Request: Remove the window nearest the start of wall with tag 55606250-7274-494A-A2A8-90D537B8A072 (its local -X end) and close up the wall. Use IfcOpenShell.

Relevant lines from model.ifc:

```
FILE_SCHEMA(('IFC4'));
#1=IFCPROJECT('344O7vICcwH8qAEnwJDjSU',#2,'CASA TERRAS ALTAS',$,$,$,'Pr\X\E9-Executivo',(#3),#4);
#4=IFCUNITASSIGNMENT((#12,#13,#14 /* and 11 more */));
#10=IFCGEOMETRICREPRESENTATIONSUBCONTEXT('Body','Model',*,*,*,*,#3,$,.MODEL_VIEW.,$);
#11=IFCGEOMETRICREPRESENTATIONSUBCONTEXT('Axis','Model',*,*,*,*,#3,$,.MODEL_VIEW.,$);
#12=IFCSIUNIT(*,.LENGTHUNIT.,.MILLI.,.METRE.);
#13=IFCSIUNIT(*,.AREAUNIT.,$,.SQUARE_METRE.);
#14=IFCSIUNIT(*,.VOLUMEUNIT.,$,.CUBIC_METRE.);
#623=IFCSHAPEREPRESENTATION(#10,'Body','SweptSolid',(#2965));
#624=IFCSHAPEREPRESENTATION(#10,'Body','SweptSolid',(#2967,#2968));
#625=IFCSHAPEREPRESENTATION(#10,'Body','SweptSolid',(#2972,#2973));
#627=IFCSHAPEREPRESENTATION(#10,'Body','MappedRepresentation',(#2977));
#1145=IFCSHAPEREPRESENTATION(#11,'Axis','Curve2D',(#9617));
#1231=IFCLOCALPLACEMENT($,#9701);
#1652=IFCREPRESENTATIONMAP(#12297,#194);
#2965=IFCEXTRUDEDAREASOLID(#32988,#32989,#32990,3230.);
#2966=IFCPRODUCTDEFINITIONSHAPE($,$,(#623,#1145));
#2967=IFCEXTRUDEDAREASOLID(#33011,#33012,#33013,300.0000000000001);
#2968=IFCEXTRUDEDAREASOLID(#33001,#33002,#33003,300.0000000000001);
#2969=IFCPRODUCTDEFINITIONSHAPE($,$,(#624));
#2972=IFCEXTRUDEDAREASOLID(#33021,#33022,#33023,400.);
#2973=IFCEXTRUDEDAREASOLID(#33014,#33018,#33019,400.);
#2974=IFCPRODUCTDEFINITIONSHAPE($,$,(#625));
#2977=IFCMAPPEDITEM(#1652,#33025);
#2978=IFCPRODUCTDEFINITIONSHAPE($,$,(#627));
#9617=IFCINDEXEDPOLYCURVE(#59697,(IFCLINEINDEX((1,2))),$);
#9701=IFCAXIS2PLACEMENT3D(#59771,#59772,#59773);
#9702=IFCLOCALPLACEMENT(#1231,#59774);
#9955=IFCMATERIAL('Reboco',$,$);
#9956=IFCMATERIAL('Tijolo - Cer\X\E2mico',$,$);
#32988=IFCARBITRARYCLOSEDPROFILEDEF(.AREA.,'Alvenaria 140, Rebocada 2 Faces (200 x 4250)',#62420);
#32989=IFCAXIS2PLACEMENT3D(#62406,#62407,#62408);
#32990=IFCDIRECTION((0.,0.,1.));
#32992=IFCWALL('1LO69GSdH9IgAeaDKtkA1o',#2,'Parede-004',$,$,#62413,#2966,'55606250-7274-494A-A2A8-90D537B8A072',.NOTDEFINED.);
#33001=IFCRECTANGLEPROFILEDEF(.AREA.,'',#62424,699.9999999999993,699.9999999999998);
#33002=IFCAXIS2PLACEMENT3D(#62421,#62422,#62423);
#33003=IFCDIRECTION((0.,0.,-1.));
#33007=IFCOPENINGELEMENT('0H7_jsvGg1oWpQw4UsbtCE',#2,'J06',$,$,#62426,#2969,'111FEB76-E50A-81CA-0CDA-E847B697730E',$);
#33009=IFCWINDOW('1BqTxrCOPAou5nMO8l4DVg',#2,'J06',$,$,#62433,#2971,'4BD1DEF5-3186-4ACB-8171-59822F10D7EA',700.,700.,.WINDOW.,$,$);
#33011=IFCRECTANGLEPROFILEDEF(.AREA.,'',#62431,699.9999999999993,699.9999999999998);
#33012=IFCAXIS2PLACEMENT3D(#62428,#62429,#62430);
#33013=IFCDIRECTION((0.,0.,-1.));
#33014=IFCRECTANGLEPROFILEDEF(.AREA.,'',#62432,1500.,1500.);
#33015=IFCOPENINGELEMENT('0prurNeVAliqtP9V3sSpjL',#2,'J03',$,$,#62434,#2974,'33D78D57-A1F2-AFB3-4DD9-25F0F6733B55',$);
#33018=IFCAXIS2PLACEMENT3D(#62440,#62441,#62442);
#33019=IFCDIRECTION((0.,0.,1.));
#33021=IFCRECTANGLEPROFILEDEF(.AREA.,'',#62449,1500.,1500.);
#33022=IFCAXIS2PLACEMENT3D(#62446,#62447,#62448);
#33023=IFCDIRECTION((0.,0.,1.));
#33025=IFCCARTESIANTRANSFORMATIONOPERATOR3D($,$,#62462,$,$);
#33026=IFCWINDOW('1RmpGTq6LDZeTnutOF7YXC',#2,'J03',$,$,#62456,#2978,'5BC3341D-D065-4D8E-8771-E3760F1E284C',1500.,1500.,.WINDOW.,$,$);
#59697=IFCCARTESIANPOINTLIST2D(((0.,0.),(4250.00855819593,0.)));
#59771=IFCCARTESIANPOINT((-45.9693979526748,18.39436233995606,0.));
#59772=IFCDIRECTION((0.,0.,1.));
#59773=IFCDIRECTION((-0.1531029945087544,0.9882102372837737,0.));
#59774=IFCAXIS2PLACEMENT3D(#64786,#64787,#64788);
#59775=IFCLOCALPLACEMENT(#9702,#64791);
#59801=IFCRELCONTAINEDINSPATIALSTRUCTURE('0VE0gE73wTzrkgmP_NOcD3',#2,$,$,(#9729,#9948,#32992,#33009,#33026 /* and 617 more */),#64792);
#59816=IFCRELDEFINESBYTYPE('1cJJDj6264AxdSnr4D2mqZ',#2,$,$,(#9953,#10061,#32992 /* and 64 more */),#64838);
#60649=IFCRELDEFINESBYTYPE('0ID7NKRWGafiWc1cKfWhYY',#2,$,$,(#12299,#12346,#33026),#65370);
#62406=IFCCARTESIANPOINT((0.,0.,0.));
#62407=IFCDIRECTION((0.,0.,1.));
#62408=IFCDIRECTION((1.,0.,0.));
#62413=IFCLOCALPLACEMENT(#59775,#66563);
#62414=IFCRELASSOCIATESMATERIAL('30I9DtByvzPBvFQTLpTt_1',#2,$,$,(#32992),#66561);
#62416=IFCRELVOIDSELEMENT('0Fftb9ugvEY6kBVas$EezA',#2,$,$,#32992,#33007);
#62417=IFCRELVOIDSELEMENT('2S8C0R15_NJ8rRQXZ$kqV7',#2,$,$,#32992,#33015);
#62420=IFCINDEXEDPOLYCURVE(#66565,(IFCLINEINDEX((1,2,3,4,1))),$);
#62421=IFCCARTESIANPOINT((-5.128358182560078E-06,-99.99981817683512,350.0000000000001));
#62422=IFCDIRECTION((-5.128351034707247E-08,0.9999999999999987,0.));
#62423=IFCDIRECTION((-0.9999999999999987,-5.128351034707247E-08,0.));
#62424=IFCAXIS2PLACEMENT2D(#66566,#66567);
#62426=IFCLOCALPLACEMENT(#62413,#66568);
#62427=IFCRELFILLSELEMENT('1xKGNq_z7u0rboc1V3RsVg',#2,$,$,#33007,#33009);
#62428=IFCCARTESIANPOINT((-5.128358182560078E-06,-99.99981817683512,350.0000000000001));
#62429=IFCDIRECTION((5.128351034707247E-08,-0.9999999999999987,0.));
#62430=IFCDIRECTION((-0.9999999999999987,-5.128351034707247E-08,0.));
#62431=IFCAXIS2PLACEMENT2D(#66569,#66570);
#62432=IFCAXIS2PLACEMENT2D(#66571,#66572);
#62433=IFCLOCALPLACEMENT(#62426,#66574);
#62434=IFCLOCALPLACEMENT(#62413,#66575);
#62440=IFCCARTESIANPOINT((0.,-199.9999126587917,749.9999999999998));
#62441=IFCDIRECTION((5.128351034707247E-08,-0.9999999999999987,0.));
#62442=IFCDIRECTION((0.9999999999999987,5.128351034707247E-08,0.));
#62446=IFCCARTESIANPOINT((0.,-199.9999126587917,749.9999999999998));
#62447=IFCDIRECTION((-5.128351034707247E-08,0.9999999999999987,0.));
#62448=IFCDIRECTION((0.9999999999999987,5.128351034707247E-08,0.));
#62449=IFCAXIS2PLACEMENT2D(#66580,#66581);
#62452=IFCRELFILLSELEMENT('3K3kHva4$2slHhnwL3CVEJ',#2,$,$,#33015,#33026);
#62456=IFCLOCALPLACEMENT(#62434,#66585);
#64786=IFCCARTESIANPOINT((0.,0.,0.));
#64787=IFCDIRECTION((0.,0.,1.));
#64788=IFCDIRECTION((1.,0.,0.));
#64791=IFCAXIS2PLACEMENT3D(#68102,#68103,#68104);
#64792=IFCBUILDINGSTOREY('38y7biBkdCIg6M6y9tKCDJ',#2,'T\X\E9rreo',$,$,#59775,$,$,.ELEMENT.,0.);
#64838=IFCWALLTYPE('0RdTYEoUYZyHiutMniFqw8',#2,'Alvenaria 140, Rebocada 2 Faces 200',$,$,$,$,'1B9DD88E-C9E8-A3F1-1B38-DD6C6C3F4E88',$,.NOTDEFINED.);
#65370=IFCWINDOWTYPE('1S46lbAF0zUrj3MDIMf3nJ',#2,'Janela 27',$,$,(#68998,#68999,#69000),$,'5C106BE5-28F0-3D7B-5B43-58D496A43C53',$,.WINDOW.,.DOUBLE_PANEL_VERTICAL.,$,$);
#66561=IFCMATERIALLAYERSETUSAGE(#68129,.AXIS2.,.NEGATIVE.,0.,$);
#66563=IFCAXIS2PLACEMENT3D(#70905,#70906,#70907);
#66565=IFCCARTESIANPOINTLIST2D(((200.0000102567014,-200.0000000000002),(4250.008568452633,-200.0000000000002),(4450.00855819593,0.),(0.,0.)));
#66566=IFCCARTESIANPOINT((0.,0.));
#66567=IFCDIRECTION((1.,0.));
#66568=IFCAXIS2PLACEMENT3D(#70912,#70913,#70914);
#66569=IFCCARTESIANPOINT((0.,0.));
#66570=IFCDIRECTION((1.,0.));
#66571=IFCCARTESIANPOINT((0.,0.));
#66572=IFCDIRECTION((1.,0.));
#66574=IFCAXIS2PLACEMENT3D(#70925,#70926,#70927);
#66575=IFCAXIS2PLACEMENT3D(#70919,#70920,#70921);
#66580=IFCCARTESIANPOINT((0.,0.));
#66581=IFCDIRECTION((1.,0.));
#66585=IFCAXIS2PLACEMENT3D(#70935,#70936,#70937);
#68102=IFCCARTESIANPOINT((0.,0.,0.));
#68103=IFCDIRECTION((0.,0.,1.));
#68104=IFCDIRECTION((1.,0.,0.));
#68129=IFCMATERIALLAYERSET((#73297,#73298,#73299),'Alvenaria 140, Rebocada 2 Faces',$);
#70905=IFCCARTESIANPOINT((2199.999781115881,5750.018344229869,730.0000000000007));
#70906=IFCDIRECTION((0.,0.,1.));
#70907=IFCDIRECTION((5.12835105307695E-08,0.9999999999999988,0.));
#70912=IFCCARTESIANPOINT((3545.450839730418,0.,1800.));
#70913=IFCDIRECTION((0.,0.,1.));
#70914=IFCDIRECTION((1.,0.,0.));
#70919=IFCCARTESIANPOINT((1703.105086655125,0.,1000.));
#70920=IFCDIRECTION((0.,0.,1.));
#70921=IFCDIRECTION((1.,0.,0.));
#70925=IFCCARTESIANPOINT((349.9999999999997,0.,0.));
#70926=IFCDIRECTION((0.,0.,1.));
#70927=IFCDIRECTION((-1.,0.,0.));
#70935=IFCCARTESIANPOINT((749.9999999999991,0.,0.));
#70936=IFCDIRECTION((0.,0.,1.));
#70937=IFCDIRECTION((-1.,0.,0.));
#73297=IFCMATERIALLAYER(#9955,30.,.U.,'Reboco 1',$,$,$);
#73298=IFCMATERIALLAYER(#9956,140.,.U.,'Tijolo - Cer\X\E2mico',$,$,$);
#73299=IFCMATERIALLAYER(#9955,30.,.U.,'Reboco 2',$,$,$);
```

```python
import ifcopenshell
import ifcopenshell.api.feature
import ifcopenshell.api.root
import ifcopenshell.geom
import ifcopenshell.util.shape

model = ifcopenshell.open("model.ifc")
settings = ifcopenshell.geom.settings()


def volume(element):
    """Net volume in cubic metres, openings subtracted."""
    shape = ifcopenshell.geom.create_shape(settings, element)
    return ifcopenshell.util.shape.get_volume(shape.geometry)


window = model.by_id(33026)
opening = window.FillsVoids[0].RelatingOpeningElement
wall = opening.VoidsElements[0].RelatingBuildingElement
before = volume(wall)

ifcopenshell.api.root.remove_product(model, product=window)
ifcopenshell.api.feature.remove_feature(model, feature=opening)

after = volume(wall)

print(f"wall volume {before:.3f} -> {after:.3f} m3")

model.write("model_rev.ifc")
```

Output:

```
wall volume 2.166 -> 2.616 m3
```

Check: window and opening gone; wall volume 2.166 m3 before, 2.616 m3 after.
